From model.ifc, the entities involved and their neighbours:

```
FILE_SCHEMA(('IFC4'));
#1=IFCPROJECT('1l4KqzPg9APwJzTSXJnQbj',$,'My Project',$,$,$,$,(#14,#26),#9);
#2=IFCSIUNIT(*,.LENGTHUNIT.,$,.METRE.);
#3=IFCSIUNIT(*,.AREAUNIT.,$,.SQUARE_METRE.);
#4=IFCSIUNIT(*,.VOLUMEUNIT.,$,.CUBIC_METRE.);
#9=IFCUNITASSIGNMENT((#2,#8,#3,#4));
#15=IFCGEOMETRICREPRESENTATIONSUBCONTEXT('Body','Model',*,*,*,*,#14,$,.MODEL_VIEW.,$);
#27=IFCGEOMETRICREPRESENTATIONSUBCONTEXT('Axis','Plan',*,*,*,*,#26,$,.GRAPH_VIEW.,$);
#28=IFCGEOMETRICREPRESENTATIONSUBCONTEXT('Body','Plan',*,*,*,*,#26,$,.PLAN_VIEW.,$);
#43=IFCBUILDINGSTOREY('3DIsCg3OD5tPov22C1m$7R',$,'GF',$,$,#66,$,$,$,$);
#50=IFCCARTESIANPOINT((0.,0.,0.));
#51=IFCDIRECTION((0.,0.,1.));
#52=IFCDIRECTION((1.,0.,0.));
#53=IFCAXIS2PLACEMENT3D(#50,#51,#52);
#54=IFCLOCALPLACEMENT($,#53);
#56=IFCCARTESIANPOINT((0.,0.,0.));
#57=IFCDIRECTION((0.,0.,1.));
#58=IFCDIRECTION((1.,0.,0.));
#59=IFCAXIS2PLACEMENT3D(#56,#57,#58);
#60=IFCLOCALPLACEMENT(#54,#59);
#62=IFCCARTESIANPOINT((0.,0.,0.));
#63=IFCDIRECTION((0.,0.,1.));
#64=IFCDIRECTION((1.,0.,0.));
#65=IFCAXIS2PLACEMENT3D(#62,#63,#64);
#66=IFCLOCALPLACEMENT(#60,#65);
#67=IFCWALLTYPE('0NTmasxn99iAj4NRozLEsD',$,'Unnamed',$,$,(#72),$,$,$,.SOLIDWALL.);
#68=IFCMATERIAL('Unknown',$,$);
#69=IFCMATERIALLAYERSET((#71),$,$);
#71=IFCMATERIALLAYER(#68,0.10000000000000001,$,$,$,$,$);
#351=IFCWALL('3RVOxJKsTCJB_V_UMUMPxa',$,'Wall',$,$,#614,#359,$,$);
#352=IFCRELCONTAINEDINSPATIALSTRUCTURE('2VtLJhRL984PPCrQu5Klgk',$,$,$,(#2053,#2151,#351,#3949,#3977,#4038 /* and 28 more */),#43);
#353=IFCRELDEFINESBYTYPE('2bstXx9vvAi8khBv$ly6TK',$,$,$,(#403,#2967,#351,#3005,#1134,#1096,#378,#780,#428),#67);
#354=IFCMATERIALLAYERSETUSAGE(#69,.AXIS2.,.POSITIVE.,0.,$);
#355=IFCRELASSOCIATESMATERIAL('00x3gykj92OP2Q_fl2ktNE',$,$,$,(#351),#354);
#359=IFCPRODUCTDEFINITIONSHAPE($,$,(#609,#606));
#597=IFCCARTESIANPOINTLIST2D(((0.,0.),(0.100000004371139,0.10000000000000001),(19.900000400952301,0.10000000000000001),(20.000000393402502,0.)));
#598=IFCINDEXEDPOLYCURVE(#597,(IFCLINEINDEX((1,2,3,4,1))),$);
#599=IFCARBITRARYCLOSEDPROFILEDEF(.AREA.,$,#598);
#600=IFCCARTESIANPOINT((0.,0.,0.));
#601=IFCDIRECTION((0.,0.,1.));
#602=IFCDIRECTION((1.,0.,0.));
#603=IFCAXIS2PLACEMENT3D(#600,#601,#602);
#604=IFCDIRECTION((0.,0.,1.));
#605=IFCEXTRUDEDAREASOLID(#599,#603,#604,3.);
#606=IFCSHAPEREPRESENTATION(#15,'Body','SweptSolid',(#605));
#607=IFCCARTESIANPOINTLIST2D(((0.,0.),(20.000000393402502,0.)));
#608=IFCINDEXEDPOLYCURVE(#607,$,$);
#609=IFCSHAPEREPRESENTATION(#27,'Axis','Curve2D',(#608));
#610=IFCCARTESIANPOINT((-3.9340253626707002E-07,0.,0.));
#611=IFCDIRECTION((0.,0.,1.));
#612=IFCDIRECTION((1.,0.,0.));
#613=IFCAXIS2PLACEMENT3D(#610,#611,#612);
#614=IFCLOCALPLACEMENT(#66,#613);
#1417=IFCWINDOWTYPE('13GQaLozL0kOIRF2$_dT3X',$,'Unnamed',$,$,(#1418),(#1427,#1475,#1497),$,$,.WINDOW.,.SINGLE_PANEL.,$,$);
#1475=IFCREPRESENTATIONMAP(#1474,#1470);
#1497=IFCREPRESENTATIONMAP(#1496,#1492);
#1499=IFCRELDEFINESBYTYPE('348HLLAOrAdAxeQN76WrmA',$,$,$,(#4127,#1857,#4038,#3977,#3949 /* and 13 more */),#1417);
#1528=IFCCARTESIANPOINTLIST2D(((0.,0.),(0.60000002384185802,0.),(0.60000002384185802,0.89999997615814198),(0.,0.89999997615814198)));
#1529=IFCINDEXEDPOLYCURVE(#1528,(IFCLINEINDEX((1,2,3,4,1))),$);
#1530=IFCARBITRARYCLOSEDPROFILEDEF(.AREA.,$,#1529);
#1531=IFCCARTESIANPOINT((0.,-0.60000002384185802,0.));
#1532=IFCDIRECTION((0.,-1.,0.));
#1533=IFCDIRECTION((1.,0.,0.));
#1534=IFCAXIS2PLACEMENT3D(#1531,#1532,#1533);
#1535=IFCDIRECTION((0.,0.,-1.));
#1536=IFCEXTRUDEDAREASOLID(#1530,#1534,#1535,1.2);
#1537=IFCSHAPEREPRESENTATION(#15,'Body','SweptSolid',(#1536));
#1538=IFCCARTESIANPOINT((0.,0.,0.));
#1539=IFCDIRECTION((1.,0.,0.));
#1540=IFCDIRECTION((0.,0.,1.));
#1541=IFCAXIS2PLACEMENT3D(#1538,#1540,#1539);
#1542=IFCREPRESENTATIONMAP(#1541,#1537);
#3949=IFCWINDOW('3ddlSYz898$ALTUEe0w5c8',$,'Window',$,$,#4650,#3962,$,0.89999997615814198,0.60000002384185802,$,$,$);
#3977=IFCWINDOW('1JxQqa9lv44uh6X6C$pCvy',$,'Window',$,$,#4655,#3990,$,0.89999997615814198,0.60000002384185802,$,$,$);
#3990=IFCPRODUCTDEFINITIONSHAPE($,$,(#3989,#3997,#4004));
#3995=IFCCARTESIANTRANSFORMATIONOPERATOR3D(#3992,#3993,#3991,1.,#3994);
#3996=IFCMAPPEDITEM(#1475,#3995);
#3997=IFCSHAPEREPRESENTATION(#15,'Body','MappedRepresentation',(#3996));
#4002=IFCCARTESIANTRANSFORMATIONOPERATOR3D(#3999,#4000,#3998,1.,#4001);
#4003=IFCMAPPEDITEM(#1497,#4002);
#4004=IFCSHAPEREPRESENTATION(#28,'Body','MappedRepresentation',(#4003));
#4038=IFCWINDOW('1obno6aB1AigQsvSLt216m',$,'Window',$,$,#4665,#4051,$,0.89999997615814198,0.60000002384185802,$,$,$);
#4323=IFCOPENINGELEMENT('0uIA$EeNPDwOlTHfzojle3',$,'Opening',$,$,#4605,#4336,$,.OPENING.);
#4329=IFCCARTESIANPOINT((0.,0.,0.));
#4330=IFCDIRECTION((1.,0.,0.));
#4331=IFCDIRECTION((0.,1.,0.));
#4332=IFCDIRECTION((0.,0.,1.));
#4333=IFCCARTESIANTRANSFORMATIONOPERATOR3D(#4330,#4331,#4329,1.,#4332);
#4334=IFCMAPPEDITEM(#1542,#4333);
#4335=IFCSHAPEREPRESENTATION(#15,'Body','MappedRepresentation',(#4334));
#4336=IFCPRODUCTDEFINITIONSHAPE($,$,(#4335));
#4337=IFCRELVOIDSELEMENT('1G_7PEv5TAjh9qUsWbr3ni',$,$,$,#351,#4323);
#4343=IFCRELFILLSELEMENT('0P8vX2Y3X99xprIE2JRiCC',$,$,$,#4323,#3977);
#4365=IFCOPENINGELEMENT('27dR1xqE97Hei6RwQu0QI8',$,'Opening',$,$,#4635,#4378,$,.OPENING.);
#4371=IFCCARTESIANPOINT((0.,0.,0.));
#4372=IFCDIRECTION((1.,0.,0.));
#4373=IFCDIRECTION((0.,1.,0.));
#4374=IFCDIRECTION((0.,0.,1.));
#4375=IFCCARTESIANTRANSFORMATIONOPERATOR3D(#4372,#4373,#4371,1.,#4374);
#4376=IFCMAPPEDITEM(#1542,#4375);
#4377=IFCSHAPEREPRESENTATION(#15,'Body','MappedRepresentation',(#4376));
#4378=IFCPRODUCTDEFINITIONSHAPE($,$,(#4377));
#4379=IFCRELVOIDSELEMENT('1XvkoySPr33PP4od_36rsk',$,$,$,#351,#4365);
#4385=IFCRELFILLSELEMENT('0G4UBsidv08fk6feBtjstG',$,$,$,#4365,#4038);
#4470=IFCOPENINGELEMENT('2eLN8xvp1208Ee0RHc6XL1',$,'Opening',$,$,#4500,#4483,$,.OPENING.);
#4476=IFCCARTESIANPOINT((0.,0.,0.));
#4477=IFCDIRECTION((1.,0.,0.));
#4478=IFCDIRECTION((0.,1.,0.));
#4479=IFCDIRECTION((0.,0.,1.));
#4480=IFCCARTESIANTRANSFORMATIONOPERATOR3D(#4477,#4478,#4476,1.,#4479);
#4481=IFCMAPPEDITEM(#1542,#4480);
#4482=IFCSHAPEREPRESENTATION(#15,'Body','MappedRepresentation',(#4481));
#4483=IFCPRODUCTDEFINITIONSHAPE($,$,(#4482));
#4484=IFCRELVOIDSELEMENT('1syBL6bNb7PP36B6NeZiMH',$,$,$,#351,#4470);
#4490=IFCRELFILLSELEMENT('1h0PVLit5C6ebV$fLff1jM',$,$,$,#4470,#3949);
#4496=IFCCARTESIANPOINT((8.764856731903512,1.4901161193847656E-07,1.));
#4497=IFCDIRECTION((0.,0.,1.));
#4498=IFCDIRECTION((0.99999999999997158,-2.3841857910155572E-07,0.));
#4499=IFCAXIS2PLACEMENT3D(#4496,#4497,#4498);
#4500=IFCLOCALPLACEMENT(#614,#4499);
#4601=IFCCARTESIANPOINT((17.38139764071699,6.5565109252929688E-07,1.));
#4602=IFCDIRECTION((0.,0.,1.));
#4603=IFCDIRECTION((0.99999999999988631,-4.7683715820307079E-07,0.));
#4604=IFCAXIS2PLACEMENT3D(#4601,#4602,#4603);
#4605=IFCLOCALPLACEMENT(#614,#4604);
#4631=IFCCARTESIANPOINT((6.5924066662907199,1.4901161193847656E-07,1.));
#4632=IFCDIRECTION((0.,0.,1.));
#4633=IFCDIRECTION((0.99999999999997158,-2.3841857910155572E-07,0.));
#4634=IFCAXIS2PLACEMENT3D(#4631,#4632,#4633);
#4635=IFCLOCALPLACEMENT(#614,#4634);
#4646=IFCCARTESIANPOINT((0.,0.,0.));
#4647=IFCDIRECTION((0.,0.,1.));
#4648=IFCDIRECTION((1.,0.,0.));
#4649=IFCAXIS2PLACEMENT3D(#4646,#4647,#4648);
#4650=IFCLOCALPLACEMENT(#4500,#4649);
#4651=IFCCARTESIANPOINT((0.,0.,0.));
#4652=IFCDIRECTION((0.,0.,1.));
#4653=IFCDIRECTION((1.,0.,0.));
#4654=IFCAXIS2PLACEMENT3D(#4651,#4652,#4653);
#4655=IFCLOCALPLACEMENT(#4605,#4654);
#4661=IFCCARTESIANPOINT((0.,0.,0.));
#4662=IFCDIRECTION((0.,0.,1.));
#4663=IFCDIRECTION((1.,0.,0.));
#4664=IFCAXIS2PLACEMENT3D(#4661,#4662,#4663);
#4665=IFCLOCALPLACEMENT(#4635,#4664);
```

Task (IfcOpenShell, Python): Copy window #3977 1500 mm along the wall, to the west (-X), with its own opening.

```python
import ifcopenshell
import ifcopenshell.api.feature
import ifcopenshell.api.geometry
import ifcopenshell.api.root
import ifcopenshell.geom
import ifcopenshell.util.element
import ifcopenshell.util.placement
import ifcopenshell.util.shape
import ifcopenshell.util.unit

model = ifcopenshell.open("model.ifc")
unit_scale = ifcopenshell.util.unit.calculate_unit_scale(model)
settings = ifcopenshell.geom.settings()


def volume(element):
    """Net volume in cubic metres, openings subtracted."""
    shape = ifcopenshell.geom.create_shape(settings, element)
    return ifcopenshell.util.shape.get_volume(shape.geometry)


window = model.by_guid("1JxQqa9lv44uh6X6C$pCvy")
opening = window.FillsVoids[0].RelatingOpeningElement
wall = opening.VoidsElements[0].RelatingBuildingElement
before = volume(wall)
shift = ifcopenshell.util.placement.get_local_placement(wall.ObjectPlacement)[:3, 0] * -1.5 / unit_scale

# copy_class copies the void relationship, type, container and properties, but no geometry.
new_opening = ifcopenshell.api.root.copy_class(model, product=opening)
new_opening.Representation = ifcopenshell.util.element.copy_deep(
    model, opening.Representation, exclude=["IfcGeometricRepresentationContext", "IfcRepresentationMap"]
)
new_window = ifcopenshell.api.root.copy_class(model, product=window)
new_window.Representation = ifcopenshell.util.element.copy_deep(
    model, window.Representation, exclude=["IfcGeometricRepresentationContext", "IfcRepresentationMap"]
)
ifcopenshell.api.feature.add_filling(model, opening=new_opening, element=new_window)

for old, new in ((opening, new_opening), (window, new_window)):
    matrix = ifcopenshell.util.placement.get_local_placement(old.ObjectPlacement)
    matrix[:3, 3] += shift
    ifcopenshell.api.geometry.edit_object_placement(model, product=new, matrix=matrix, is_si=False)

after = volume(wall)

print(f"wall volume {before:.3f} -> {after:.3f} m3")

model.write("model_v2.ifc")
```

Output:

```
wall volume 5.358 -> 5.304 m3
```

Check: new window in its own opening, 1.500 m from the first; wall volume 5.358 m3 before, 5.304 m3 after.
